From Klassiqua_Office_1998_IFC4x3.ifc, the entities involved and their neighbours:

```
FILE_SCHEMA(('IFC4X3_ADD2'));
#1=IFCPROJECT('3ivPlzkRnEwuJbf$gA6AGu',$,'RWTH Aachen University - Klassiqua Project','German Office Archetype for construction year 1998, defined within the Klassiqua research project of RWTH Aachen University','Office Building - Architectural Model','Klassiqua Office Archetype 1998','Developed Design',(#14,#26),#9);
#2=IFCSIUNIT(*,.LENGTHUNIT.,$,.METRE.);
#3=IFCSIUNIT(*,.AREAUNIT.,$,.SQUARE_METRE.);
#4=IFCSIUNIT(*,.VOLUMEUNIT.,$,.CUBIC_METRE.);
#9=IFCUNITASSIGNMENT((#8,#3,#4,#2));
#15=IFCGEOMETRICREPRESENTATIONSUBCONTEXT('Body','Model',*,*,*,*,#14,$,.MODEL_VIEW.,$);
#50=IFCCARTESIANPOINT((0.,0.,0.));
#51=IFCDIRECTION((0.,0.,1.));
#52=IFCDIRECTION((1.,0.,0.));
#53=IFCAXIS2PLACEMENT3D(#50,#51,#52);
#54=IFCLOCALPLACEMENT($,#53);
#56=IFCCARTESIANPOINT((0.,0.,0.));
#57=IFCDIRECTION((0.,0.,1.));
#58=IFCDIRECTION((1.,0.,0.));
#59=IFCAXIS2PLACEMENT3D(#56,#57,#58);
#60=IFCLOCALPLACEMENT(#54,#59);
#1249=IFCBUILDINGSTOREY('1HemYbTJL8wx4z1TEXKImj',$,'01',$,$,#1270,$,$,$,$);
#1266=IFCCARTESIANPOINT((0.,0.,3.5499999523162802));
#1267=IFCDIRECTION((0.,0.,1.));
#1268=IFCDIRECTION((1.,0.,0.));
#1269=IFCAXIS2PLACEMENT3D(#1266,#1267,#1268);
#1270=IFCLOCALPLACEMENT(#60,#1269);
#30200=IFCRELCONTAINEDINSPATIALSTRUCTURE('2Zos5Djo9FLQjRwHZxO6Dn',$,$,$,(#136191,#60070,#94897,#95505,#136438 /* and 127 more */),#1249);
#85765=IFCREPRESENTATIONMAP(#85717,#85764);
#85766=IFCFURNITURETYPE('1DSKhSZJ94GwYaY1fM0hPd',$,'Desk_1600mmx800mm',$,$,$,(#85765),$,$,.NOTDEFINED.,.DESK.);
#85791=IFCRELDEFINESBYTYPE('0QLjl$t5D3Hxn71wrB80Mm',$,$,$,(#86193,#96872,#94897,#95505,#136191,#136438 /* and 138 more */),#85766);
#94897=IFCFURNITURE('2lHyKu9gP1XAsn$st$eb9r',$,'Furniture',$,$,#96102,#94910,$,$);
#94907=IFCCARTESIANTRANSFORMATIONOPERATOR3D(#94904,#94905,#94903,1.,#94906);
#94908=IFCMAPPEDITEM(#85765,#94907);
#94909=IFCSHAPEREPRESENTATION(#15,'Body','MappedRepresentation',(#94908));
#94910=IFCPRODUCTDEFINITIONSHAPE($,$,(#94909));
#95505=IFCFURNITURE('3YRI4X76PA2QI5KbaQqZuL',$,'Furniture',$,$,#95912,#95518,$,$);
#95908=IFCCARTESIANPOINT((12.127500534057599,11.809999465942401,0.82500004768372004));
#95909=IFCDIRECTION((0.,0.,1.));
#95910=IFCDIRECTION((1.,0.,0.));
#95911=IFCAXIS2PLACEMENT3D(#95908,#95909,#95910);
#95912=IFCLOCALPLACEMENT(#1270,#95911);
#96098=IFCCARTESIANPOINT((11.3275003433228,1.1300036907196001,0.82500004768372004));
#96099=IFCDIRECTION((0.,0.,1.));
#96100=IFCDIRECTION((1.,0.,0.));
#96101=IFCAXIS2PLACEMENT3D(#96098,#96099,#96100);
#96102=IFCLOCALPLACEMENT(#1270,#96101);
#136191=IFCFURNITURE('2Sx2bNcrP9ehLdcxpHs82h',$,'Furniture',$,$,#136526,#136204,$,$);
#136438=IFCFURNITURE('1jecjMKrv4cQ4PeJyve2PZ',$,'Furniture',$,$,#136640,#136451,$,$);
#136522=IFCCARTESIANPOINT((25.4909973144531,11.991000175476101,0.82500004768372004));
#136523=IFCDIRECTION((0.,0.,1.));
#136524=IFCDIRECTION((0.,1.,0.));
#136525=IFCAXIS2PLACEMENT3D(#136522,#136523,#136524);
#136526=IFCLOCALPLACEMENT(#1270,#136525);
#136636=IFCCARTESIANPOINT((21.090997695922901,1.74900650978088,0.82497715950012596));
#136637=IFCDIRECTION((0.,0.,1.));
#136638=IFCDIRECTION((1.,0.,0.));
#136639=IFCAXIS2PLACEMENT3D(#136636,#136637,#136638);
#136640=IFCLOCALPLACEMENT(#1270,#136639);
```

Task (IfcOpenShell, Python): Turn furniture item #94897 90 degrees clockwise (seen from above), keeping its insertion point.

```python
import ifcopenshell
import ifcopenshell.api.geometry
import ifcopenshell.util.placement

model = ifcopenshell.open("Klassiqua_Office_1998_IFC4x3.ifc")

item = model.by_guid("2lHyKu9gP1XAsn$st$eb9r")
matrix = ifcopenshell.util.placement.get_local_placement(item.ObjectPlacement)
matrix = matrix @ ifcopenshell.util.placement.rotation(-90, "Z")
ifcopenshell.api.geometry.edit_object_placement(model, product=item, matrix=matrix, is_si=False)

print(ifcopenshell.util.placement.get_local_placement(item.ObjectPlacement).round(3) + 0.0)

model.write("Klassiqua_Office_1998_IFC4x3_edited.ifc")
```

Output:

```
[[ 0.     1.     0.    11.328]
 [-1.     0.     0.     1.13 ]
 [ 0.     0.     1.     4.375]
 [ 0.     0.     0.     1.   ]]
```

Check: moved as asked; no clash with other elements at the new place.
